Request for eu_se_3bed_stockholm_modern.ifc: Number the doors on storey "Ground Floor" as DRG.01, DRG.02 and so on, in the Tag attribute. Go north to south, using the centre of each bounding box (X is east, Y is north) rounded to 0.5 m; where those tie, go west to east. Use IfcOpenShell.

First a look at what the model holds.

```python
import ifcopenshell
import ifcopenshell.util.element
import ifcopenshell.util.placement

model = ifcopenshell.open("eu_se_3bed_stockholm_modern.ifc")
print(model.schema)
storey = next(s for s in model.by_type("IfcBuildingStorey") if s.Name == "Ground Floor")
doors = [e for e in ifcopenshell.util.element.get_decomposition(storey) if e.is_a("IfcDoor")]
for e in sorted(doors, key=lambda e: e.id()):
    origin = ifcopenshell.util.placement.get_local_placement(e.ObjectPlacement)[:3, 3]
    print(e.id(), e.Tag, e.Name, origin.round(2) + 0.0, sep=" | ")
```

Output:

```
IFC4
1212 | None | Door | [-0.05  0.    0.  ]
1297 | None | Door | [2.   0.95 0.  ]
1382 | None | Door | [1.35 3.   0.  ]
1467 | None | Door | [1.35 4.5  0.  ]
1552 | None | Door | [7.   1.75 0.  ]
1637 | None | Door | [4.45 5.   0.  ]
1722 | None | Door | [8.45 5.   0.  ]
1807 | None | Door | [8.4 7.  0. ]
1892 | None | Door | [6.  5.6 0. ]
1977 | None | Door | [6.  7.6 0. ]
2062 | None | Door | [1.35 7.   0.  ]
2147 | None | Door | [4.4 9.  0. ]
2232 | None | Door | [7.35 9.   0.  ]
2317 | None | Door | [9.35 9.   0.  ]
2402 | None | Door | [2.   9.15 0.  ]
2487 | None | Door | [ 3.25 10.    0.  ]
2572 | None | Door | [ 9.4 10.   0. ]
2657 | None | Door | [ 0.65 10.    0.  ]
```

```python
import ifcopenshell
import ifcopenshell.geom
import ifcopenshell.util.element
import ifcopenshell.util.shape

model = ifcopenshell.open("eu_se_3bed_stockholm_modern.ifc")
settings = ifcopenshell.geom.settings()
settings.set("use-world-coords", True)


def centre(element):
    shape = ifcopenshell.geom.create_shape(settings, element)
    return ifcopenshell.util.shape.get_bbox_centroid(shape.geometry)


storey = next(s for s in model.by_type("IfcBuildingStorey") if s.Name == "Ground Floor")
doors = [e for e in ifcopenshell.util.element.get_decomposition(storey) if e.is_a("IfcDoor")]

# Insertion points can sit at a corner or the storey origin, so sort by the geometry (in metres).
centres = {e: centre(e) for e in doors}
doors.sort(key=lambda e: (-round(centres[e][1] / 0.5), centres[e][0]))

for i, e in enumerate(doors, start=1):
    number = f"DRG.{i:02d}"
    e.Tag = number
    print(e.id(), number)

model.write("eu_se_3bed_stockholm_modern-out.ifc")
```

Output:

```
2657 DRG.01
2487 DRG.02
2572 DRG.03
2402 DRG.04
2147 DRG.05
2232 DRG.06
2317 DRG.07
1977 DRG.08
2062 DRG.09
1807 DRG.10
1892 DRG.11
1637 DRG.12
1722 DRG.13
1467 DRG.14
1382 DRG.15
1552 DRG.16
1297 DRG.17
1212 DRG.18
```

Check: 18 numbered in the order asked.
